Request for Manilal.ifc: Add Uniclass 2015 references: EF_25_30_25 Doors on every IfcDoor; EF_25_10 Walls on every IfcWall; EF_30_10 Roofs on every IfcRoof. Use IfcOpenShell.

First a look at what the model holds.

```python
import ifcopenshell

model = ifcopenshell.open("Manilal.ifc")
print(model.schema)
print("classifications:", [c.Name for c in model.by_type("IfcClassification")])
for ifc_class in ("IfcDoor", "IfcRoof", "IfcStair", "IfcWall", "IfcWindow"):
    print(ifc_class, len(model.by_type(ifc_class)))
```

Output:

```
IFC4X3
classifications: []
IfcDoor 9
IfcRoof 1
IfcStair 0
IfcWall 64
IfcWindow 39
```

```python
import ifcopenshell
import ifcopenshell.api.classification

model = ifcopenshell.open("Manilal.ifc")

system = ifcopenshell.api.classification.add_classification(model, classification="Uniclass 2015")

codes = {
    "IfcDoor": ("EF_25_30_25", "Doors"),
    "IfcWall": ("EF_25_10", "Walls"),
    "IfcRoof": ("EF_30_10", "Roofs"),
}
for ifc_class, (code, name) in codes.items():
    products = model.by_type(ifc_class)
    ifcopenshell.api.classification.add_reference(
        model, products=products, classification=system, identification=code, name=name
    )
    print(code, len(products))

model.write("Manilal_v2.ifc")
```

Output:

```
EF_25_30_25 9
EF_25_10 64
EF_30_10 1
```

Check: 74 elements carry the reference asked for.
